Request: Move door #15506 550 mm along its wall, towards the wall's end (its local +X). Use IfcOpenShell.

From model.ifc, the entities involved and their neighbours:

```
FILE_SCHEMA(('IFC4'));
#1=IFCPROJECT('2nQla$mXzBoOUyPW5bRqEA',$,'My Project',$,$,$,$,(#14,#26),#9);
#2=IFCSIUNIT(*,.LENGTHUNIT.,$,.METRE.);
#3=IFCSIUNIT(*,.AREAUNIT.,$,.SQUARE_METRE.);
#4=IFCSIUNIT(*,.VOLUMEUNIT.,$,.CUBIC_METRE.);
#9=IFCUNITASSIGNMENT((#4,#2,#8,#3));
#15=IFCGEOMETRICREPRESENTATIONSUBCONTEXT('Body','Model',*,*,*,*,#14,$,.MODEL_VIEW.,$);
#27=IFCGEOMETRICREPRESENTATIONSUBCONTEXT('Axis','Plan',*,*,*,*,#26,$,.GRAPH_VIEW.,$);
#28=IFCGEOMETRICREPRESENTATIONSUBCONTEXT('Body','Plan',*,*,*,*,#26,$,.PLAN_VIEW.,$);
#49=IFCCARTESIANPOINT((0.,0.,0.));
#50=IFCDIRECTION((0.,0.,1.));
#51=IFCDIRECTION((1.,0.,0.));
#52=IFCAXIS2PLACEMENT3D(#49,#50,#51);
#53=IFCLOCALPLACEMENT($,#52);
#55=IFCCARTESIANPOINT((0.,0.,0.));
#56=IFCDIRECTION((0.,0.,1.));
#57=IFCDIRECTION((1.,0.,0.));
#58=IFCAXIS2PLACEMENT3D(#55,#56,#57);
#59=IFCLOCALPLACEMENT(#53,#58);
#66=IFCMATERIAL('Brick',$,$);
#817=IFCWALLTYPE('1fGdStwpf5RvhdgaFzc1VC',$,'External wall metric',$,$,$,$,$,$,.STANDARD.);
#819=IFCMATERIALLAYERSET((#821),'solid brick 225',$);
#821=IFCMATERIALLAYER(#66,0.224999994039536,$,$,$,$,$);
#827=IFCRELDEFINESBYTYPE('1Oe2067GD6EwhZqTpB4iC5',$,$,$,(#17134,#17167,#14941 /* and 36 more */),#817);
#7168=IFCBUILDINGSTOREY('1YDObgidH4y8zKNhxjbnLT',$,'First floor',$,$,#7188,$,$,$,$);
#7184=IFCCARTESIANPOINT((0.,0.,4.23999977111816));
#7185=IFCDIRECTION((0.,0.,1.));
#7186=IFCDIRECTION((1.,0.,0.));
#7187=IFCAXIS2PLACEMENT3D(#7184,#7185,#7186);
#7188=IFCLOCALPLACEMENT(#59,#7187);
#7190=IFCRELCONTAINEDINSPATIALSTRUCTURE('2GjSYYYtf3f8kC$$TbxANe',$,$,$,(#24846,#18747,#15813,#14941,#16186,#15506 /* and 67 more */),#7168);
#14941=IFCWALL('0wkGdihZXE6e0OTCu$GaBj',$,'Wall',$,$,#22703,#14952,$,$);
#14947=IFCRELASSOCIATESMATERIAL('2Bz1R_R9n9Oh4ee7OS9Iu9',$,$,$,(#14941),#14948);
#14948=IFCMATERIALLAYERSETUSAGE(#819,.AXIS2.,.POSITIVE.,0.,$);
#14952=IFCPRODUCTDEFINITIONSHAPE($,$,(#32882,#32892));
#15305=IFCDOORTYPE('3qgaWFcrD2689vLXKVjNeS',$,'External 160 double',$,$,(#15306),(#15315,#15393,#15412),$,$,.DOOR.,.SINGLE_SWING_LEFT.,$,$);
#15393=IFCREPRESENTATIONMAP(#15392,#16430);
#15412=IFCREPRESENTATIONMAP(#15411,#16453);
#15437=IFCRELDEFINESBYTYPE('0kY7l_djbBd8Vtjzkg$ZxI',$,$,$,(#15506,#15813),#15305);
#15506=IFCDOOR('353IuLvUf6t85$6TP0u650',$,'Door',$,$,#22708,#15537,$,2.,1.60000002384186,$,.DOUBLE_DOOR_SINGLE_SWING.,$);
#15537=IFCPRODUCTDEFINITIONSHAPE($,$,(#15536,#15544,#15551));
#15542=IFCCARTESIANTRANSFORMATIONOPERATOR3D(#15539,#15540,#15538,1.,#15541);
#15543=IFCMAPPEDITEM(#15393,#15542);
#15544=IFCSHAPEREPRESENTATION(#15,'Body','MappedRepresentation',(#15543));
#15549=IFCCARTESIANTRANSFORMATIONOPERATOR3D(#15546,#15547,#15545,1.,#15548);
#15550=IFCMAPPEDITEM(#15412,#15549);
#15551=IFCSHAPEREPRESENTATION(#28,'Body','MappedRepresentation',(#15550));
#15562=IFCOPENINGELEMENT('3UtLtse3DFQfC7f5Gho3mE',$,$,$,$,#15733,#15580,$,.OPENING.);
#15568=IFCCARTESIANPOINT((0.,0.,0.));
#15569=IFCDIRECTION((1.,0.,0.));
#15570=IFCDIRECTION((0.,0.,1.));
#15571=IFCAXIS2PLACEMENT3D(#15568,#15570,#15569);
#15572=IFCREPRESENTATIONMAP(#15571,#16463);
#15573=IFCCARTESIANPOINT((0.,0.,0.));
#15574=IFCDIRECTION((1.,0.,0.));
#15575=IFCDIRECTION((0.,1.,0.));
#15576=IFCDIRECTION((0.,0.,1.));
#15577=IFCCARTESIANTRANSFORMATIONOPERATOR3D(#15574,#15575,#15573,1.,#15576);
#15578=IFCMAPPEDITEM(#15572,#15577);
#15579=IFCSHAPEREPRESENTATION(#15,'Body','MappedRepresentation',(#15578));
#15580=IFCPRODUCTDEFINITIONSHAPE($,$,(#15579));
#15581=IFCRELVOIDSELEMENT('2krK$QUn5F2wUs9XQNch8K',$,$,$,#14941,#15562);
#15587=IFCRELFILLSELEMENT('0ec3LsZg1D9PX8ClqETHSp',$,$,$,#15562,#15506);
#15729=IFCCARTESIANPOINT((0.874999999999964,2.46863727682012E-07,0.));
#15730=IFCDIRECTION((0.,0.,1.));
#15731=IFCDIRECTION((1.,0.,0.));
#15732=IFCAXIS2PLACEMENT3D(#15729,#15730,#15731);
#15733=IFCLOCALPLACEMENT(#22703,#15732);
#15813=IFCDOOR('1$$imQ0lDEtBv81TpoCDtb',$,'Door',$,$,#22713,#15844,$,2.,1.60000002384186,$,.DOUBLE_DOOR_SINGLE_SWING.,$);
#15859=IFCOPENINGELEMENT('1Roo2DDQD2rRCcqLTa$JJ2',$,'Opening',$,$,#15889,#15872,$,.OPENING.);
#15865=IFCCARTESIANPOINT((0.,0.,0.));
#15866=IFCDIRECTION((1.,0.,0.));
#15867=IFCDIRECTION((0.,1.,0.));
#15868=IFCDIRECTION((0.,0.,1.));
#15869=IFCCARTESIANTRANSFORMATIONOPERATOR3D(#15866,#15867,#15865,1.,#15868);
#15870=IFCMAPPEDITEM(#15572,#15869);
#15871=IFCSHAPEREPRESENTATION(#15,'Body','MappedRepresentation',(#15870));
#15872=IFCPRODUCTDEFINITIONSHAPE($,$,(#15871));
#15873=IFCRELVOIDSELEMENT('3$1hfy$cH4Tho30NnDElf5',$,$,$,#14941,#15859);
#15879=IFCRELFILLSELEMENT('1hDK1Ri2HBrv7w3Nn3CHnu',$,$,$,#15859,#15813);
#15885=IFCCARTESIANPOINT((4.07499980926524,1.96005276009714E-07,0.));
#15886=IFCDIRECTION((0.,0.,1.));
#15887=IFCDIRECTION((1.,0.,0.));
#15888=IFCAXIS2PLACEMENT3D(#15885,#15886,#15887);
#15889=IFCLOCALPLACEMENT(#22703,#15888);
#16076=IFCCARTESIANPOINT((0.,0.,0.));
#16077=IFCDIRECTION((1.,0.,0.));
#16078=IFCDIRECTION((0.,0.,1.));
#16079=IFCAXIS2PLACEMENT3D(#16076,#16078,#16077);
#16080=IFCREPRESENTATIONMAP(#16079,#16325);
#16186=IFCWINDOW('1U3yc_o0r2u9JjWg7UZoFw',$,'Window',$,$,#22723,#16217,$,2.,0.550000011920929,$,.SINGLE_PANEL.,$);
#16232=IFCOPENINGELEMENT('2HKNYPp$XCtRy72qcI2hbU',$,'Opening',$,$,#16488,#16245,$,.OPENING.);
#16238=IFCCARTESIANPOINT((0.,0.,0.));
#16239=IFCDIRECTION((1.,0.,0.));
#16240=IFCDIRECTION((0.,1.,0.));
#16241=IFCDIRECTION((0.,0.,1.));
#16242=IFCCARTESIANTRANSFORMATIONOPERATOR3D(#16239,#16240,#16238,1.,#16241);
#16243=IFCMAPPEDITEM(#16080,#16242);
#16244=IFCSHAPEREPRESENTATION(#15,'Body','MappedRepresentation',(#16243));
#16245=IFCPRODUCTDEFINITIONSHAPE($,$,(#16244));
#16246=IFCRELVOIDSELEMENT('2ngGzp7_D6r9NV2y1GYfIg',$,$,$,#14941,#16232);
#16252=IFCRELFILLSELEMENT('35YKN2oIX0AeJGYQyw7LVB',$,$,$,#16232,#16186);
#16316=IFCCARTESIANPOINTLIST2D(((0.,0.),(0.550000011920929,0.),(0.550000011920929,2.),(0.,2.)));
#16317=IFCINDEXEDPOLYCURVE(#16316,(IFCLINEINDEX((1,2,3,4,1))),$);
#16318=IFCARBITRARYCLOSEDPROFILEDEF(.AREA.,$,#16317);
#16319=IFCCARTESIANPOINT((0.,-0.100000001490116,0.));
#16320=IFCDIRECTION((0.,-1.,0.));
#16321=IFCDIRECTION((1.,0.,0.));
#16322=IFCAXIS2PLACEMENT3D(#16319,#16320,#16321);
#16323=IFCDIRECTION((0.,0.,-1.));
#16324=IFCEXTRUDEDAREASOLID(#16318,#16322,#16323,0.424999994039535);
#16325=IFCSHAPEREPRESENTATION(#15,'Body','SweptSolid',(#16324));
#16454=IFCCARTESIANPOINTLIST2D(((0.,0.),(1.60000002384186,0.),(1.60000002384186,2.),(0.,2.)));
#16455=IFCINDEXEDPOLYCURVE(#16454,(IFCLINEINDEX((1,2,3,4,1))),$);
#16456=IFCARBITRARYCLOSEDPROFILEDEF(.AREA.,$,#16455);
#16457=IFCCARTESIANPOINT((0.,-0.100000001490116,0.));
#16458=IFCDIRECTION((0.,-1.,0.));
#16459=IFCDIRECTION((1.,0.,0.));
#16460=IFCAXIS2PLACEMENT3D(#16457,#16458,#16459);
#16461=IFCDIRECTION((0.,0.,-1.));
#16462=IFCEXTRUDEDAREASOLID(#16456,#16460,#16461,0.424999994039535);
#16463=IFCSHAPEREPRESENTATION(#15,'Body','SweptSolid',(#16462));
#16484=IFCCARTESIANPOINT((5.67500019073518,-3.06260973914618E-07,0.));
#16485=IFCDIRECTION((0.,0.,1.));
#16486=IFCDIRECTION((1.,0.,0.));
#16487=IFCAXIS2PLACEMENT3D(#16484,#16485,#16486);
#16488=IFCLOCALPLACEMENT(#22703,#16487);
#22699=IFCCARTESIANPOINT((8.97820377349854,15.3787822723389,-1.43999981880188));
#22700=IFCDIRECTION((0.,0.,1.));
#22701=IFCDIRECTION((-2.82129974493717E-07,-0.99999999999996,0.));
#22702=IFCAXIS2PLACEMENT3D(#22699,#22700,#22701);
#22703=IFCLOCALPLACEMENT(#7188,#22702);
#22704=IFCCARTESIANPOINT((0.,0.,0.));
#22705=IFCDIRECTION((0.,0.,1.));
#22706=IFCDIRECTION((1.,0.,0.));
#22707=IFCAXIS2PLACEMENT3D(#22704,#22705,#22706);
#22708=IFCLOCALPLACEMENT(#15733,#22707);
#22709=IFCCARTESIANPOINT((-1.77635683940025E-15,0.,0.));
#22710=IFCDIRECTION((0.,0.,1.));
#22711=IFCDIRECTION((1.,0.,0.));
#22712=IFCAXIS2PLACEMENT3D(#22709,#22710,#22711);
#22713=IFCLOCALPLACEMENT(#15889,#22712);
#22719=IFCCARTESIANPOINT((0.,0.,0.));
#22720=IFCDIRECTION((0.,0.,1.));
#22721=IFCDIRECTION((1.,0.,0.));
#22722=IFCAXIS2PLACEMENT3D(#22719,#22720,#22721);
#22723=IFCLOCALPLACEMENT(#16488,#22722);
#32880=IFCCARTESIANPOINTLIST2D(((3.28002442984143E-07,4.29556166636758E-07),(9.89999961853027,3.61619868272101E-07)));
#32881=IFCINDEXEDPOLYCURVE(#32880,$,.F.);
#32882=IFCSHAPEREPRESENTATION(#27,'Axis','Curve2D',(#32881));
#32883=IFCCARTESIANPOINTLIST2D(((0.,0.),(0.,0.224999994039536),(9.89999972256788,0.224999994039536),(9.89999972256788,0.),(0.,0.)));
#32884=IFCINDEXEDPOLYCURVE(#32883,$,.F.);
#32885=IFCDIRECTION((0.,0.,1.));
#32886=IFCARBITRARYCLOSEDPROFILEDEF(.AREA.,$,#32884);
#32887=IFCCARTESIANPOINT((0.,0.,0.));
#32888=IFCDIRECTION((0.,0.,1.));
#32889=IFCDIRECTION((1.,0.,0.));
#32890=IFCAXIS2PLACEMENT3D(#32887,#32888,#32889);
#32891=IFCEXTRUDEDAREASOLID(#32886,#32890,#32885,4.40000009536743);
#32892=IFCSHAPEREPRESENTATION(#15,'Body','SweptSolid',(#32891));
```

```python
import ifcopenshell
import ifcopenshell.api.geometry
import ifcopenshell.util.placement
import ifcopenshell.util.unit

model = ifcopenshell.open("model.ifc")
unit_scale = ifcopenshell.util.unit.calculate_unit_scale(model)

door = model.by_guid("353IuLvUf6t85$6TP0u650")
opening = door.FillsVoids[0].RelatingOpeningElement
wall = opening.VoidsElements[0].RelatingBuildingElement

wall_matrix = ifcopenshell.util.placement.get_local_placement(wall.ObjectPlacement)
shift = wall_matrix[:3, 0] * 0.55 / unit_scale
before = ifcopenshell.util.placement.get_local_placement(door.ObjectPlacement)[:3, 3].copy()

# The door is placed relative to its opening, so it follows when the opening moves.
matrix = ifcopenshell.util.placement.get_local_placement(opening.ObjectPlacement)
matrix[:3, 3] += shift
ifcopenshell.api.geometry.edit_object_placement(
    model, product=opening, matrix=matrix, is_si=False, should_transform_children=True
)

after = ifcopenshell.util.placement.get_local_placement(door.ObjectPlacement)[:3, 3]
print("door moved by", (after - before).round(3) + 0.0)

model.write("model-out.ifc")
```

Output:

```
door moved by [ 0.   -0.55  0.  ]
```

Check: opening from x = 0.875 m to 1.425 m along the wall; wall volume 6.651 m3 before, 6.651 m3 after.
